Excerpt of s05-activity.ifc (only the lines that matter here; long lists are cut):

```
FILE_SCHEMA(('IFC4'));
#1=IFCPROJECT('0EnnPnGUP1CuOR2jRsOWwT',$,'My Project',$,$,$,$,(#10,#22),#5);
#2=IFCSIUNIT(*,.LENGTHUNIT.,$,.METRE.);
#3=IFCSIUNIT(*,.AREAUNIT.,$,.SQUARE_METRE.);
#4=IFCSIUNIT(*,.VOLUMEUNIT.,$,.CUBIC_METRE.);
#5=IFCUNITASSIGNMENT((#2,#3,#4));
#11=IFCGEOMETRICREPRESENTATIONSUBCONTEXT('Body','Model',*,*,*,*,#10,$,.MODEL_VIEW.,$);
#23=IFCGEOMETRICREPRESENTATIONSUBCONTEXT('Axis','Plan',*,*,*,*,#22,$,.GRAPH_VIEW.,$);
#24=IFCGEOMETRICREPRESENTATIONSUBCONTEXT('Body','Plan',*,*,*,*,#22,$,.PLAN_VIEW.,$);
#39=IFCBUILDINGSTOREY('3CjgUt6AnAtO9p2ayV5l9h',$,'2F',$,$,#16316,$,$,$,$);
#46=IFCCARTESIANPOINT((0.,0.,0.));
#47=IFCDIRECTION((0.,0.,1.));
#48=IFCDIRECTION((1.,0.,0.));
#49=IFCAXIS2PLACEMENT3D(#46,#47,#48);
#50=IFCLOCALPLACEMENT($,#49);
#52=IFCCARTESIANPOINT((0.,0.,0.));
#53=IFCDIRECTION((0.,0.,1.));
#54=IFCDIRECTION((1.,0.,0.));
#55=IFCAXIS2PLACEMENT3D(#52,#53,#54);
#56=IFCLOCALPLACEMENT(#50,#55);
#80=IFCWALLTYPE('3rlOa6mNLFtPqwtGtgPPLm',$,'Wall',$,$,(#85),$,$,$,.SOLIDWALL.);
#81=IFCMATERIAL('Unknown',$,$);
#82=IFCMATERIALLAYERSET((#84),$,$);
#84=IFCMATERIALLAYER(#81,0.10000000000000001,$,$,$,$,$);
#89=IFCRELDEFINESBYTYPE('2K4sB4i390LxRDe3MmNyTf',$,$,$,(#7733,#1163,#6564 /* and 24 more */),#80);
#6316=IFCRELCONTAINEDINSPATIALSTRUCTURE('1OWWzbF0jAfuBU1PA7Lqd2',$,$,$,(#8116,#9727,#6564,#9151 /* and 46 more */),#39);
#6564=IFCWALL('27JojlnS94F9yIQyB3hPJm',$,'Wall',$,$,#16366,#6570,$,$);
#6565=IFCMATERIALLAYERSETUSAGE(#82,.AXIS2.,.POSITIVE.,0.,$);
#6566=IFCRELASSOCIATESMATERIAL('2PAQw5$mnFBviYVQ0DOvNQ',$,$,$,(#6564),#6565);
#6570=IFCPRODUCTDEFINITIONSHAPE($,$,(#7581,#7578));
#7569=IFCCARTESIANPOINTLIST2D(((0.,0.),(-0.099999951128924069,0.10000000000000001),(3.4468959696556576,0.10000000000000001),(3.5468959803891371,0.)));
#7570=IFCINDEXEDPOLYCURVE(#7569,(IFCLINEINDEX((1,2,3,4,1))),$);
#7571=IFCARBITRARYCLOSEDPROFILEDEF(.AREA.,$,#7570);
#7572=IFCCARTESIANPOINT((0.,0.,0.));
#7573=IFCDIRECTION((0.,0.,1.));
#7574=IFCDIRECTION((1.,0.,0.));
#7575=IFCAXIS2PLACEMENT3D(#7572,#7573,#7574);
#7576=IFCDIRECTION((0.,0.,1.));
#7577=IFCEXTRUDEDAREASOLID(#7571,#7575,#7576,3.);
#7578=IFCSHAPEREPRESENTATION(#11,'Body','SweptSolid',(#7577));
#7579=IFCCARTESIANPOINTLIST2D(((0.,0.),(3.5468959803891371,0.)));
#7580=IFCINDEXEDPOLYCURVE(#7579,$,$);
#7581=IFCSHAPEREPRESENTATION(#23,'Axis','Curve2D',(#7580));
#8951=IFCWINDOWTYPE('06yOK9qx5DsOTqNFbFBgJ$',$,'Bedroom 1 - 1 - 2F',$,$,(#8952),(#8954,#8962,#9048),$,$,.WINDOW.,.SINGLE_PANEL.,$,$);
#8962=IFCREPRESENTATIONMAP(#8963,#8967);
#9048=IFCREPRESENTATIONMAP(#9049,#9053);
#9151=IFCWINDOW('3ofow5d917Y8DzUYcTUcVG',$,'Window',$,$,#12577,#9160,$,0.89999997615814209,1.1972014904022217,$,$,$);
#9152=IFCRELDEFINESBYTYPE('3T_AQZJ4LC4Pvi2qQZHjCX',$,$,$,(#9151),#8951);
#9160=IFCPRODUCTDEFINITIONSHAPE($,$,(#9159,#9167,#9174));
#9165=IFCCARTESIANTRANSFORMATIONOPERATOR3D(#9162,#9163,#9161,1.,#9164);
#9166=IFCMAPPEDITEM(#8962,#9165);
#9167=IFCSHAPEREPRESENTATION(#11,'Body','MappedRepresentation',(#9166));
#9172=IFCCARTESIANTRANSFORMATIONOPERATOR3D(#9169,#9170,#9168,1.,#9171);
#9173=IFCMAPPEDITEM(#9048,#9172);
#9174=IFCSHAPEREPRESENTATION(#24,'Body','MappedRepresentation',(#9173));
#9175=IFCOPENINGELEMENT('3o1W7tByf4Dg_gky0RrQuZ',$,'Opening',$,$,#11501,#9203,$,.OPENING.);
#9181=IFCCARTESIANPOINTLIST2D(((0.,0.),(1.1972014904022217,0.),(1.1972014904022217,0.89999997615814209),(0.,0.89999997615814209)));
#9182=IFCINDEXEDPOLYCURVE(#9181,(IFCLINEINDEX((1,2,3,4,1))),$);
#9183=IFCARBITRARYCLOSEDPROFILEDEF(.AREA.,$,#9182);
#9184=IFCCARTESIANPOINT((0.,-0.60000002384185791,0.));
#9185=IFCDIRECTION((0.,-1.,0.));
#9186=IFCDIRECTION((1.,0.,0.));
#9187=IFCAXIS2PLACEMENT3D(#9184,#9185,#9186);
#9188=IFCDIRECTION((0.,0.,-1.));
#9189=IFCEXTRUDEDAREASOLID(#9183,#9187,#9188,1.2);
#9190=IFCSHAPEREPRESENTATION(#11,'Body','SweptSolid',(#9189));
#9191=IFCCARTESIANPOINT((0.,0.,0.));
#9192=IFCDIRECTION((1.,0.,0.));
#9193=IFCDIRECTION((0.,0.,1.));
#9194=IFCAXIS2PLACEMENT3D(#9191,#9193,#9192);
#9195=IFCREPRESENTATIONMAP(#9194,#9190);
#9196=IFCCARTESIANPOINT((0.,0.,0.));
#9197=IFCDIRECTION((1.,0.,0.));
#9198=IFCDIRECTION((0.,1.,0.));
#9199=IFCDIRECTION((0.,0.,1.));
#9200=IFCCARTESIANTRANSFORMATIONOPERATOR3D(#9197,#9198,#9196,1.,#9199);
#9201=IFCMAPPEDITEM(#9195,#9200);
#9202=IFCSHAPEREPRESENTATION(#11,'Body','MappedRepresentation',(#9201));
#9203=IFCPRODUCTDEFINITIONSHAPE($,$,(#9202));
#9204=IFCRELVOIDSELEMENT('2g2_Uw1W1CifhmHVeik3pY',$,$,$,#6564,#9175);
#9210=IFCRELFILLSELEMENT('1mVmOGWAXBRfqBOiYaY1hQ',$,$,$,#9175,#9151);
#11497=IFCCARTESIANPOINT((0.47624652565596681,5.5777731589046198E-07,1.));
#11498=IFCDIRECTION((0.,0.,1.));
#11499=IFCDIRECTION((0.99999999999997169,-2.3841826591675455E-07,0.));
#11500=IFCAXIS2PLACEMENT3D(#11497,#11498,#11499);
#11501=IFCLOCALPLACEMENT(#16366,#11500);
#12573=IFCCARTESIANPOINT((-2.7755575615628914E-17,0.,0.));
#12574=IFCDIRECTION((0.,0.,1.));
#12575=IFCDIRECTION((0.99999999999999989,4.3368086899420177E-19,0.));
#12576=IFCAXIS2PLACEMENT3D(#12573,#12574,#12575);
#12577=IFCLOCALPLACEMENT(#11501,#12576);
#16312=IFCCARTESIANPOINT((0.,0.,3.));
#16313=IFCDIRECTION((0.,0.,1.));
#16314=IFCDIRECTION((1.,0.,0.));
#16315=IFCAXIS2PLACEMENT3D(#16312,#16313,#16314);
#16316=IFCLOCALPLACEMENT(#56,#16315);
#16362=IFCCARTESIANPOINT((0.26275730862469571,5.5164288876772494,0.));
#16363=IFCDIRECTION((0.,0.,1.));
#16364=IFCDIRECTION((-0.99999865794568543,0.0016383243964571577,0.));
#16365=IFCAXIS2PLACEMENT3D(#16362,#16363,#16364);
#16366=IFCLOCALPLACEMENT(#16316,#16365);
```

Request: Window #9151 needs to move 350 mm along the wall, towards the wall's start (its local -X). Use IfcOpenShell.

```python
import ifcopenshell
import ifcopenshell.api.geometry
import ifcopenshell.util.placement

model = ifcopenshell.open("s05-activity.ifc")

window = model.by_guid("3ofow5d917Y8DzUYcTUcVG")
opening = window.FillsVoids[0].RelatingOpeningElement
wall = opening.VoidsElements[0].RelatingBuildingElement

wall_matrix = ifcopenshell.util.placement.get_local_placement(wall.ObjectPlacement)
shift = wall_matrix[:3, 0] * -0.35
before = ifcopenshell.util.placement.get_local_placement(window.ObjectPlacement)[:3, 3].copy()

# The window is placed relative to its opening, so it follows when the opening moves.
matrix = ifcopenshell.util.placement.get_local_placement(opening.ObjectPlacement)
matrix[:3, 3] += shift
ifcopenshell.api.geometry.edit_object_placement(
    model, product=opening, matrix=matrix, is_si=False, should_transform_children=True
)

after = ifcopenshell.util.placement.get_local_placement(window.ObjectPlacement)[:3, 3]
print("window moved by", (after - before).round(3) + 0.0)

model.write("s05-activity-out.ifc")
```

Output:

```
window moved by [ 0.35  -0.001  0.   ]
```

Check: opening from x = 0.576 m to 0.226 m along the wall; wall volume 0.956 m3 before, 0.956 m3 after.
